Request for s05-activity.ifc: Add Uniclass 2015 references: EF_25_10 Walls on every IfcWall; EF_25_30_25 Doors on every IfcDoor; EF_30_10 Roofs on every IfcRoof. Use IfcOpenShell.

First a look at what the model holds.

```python
import ifcopenshell

model = ifcopenshell.open("s05-activity.ifc")
print(model.schema)
print("classifications:", [c.Name for c in model.by_type("IfcClassification")])
for ifc_class in ("IfcDoor", "IfcRoof", "IfcStair", "IfcWall", "IfcWindow"):
    print(ifc_class, len(model.by_type(ifc_class)))
```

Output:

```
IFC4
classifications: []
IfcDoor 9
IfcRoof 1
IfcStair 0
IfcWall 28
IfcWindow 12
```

```python
import ifcopenshell
import ifcopenshell.api.classification

model = ifcopenshell.open("s05-activity.ifc")

system = ifcopenshell.api.classification.add_classification(model, classification="Uniclass 2015")

codes = {
    "IfcWall": ("EF_25_10", "Walls"),
    "IfcDoor": ("EF_25_30_25", "Doors"),
    "IfcRoof": ("EF_30_10", "Roofs"),
}
for ifc_class, (code, name) in codes.items():
    products = model.by_type(ifc_class)
    ifcopenshell.api.classification.add_reference(
        model, products=products, classification=system, identification=code, name=name
    )
    print(code, len(products))

model.write("s05-activity_updated.ifc")
```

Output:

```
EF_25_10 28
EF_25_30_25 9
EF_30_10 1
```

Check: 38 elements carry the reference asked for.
